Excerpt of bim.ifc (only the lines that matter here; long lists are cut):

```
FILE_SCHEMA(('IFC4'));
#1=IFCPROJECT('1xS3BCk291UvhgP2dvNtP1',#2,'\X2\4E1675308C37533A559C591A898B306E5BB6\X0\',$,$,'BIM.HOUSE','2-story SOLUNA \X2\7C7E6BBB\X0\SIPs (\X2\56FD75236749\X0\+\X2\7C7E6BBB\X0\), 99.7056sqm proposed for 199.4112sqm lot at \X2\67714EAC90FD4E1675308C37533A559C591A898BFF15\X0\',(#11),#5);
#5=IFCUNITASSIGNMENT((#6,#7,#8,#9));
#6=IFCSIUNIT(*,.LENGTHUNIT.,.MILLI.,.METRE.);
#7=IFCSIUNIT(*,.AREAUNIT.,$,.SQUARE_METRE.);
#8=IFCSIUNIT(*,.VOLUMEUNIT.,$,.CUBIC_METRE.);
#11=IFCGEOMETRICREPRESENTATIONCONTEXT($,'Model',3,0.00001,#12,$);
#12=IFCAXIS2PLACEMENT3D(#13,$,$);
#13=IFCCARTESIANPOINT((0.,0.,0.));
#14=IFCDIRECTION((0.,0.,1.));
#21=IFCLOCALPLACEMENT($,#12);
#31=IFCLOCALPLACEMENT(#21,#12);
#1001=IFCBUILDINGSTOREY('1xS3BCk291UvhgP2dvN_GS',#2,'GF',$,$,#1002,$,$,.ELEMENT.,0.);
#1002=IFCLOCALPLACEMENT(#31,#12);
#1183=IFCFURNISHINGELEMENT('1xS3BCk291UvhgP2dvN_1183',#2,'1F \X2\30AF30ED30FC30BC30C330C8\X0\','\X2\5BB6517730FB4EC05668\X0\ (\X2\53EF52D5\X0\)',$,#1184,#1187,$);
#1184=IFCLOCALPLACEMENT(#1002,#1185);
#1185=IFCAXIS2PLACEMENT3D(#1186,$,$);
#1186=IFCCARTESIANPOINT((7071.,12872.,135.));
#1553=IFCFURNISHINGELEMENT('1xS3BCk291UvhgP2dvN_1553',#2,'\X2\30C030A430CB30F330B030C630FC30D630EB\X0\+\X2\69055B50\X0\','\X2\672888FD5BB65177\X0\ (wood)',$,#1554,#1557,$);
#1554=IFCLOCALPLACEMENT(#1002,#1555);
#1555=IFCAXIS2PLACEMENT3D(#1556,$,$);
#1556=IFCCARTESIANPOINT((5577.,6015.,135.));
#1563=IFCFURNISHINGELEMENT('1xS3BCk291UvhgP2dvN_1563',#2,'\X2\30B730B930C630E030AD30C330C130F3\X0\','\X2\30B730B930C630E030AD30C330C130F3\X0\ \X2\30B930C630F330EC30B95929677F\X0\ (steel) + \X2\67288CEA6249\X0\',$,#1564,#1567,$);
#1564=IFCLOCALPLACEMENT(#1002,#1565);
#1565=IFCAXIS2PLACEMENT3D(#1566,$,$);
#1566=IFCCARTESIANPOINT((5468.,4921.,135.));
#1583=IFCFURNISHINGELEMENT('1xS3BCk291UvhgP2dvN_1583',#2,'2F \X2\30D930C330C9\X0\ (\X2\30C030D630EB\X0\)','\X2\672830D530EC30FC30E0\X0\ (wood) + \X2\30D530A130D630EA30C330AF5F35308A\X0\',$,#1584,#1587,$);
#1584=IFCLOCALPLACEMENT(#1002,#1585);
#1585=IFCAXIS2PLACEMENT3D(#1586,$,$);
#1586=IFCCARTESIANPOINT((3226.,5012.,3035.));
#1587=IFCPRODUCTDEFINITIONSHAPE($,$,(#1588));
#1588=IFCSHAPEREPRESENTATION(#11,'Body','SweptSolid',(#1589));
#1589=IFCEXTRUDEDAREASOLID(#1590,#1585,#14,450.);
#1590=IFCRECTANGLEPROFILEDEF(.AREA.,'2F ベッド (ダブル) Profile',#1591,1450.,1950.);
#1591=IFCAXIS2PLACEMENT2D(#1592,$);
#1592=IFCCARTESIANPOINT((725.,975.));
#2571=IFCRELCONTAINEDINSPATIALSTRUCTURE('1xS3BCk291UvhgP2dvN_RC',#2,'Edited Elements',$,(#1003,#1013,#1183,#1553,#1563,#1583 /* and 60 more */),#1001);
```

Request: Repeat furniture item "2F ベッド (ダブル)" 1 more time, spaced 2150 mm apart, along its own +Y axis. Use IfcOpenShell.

```python
import ifcopenshell
import ifcopenshell.api.geometry
import ifcopenshell.api.root
import ifcopenshell.util.element
import ifcopenshell.util.placement

model = ifcopenshell.open("bim.ifc")


def reuse_history(source, copy):
    """copy_class also copies each property set's owner history, people and application; keep the originals."""
    for rel in copy.IsDefinedBy:
        if rel.is_a("IfcRelDefinesByProperties") and (history := rel.RelatingPropertyDefinition.OwnerHistory):
            rel.RelatingPropertyDefinition.OwnerHistory = source.OwnerHistory
            ifcopenshell.util.element.remove_deep2(model, history)


source = model.by_id(1583)
base = ifcopenshell.util.placement.get_local_placement(source.ObjectPlacement)
step = base[:3, 1] * 2150.0

for i in range(1, 2):
    copy = ifcopenshell.api.root.copy_class(model, product=source)
    copy.Representation = ifcopenshell.util.element.copy_deep(
        model, source.Representation, exclude=["IfcGeometricRepresentationContext", "IfcRepresentationMap"]
    )
    reuse_history(source, copy)
    matrix = base.copy()
    matrix[:3, 3] += i * step
    print("added at", matrix[:3, 3].round(3) + 0.0)
    ifcopenshell.api.geometry.edit_object_placement(model, product=copy, matrix=matrix, is_si=False)

model.write("bim_v2.ifc")
```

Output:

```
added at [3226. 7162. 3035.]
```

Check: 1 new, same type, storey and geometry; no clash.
